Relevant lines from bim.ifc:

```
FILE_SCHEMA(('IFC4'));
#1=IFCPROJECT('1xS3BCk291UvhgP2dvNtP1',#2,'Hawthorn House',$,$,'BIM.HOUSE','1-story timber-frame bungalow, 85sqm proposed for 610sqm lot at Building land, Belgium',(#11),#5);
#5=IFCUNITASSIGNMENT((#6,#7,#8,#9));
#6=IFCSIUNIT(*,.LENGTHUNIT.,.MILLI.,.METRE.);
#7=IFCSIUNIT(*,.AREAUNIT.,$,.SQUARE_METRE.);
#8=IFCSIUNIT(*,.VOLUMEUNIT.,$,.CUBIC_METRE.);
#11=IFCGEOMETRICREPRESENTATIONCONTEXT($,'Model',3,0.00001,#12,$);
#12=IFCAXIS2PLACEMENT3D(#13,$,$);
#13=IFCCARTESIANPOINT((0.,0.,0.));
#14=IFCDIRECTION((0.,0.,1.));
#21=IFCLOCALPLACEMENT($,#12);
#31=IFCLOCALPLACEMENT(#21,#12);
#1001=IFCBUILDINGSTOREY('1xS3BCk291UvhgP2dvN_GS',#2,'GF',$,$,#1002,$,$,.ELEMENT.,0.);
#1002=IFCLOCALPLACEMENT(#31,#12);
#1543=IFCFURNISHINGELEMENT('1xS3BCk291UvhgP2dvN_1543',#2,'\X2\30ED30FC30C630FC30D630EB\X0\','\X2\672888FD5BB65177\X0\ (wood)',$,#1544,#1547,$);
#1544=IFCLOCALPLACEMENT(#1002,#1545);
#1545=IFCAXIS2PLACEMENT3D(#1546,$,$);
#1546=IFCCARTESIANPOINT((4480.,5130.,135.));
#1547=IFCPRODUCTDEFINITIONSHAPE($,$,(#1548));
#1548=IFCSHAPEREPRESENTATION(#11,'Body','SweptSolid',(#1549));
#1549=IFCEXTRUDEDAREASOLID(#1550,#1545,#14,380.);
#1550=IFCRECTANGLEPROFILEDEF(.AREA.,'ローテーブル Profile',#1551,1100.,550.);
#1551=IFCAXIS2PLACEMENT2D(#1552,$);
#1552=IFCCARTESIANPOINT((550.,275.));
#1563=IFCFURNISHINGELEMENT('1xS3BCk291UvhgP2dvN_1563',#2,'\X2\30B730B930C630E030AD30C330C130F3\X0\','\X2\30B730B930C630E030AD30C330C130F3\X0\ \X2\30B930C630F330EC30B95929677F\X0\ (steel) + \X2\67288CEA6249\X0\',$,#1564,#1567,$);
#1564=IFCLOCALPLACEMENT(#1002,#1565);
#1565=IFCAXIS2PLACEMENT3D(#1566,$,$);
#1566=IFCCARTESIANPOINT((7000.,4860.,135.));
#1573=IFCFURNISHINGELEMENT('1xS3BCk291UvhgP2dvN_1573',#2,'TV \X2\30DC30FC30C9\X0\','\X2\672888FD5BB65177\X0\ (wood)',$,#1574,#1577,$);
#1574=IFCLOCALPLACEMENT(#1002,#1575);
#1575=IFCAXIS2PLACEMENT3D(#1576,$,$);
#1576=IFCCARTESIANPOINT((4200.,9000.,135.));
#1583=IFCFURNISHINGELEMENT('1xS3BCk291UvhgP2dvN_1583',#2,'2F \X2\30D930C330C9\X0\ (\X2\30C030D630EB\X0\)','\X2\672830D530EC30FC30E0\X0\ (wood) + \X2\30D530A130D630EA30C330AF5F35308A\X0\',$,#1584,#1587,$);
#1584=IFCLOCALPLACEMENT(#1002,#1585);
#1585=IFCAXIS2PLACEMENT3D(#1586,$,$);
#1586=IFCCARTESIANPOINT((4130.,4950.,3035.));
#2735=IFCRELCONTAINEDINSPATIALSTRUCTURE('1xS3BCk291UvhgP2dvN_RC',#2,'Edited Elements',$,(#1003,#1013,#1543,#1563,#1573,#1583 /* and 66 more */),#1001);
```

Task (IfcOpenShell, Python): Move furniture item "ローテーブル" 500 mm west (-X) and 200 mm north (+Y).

```python
import ifcopenshell
import ifcopenshell.api.geometry
import ifcopenshell.util.placement

model = ifcopenshell.open("bim.ifc")

item = model.by_id(1543)
matrix = ifcopenshell.util.placement.get_local_placement(item.ObjectPlacement)
matrix[0, 3] -= 500.0
matrix[1, 3] += 200.0
ifcopenshell.api.geometry.edit_object_placement(model, product=item, matrix=matrix, is_si=False)

print(ifcopenshell.util.placement.get_local_placement(item.ObjectPlacement).round(3) + 0.0)

model.write("bim_updated.ifc")
```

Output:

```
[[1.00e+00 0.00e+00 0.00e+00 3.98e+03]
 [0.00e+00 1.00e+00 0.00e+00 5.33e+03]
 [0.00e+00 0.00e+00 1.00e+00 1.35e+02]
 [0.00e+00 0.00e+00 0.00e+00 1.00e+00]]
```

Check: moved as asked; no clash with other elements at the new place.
